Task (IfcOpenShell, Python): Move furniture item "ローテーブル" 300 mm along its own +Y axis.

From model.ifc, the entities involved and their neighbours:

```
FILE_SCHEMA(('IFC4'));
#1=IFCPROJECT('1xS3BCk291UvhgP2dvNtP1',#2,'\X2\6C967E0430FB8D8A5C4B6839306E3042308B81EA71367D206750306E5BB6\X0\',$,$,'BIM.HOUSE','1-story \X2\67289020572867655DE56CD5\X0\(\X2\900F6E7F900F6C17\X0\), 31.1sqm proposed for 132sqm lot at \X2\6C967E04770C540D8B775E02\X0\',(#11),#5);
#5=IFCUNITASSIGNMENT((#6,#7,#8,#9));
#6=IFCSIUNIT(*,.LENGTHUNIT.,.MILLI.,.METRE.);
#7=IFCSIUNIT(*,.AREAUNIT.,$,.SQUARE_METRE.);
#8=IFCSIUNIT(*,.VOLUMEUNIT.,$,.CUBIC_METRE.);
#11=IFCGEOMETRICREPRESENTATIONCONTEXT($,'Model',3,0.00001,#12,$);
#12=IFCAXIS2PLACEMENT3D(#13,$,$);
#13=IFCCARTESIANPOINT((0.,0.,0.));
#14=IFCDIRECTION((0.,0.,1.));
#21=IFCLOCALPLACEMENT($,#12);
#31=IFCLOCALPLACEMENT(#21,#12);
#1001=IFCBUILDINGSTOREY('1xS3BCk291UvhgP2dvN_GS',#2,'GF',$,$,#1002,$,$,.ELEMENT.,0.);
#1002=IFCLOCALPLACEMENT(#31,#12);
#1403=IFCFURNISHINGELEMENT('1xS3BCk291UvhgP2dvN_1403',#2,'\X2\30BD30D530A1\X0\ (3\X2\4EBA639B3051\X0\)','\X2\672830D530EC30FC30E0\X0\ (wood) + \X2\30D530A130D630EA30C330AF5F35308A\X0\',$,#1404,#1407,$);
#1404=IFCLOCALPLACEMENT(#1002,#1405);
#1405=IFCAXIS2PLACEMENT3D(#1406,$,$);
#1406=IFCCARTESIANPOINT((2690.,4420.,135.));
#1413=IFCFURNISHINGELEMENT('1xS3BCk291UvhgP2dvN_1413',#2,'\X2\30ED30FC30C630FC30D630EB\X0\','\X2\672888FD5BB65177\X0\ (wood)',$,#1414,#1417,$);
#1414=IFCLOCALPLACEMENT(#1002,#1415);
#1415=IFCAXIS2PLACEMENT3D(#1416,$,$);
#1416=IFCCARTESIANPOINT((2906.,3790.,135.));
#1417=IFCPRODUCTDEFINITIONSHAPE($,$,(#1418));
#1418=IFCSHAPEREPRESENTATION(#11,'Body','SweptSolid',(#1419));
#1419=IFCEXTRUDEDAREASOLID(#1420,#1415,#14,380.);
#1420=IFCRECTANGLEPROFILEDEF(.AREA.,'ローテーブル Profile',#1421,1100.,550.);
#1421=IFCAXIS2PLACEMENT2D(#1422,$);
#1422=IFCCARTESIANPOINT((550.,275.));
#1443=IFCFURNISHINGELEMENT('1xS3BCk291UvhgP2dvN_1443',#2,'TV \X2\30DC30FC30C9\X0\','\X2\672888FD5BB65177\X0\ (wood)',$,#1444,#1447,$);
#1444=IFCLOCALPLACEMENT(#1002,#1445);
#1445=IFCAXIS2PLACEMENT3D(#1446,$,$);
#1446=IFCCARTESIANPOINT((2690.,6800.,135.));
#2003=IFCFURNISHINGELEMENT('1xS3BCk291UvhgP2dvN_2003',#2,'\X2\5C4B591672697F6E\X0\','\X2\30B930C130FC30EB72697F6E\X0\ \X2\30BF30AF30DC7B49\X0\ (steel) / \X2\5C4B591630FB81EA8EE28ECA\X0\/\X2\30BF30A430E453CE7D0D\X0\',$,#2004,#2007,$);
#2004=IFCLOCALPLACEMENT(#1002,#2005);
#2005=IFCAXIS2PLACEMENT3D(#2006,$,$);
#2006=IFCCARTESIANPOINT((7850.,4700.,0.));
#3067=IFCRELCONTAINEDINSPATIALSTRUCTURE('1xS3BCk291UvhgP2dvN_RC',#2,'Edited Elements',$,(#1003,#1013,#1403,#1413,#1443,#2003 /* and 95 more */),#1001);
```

```python
import ifcopenshell
import ifcopenshell.api.geometry
import ifcopenshell.util.placement

model = ifcopenshell.open("model.ifc")

item = model.by_guid("1xS3BCk291UvhgP2dvN_1413")
matrix = ifcopenshell.util.placement.get_local_placement(item.ObjectPlacement)
matrix[:3, 3] += matrix[:3, 1] * 300.0
ifcopenshell.api.geometry.edit_object_placement(model, product=item, matrix=matrix, is_si=False)

print(ifcopenshell.util.placement.get_local_placement(item.ObjectPlacement).round(3) + 0.0)

model.write("model_rev.ifc")
```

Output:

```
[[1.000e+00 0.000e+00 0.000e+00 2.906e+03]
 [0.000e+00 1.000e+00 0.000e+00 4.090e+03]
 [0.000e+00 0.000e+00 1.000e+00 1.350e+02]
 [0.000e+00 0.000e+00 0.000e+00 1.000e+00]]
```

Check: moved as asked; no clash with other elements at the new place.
